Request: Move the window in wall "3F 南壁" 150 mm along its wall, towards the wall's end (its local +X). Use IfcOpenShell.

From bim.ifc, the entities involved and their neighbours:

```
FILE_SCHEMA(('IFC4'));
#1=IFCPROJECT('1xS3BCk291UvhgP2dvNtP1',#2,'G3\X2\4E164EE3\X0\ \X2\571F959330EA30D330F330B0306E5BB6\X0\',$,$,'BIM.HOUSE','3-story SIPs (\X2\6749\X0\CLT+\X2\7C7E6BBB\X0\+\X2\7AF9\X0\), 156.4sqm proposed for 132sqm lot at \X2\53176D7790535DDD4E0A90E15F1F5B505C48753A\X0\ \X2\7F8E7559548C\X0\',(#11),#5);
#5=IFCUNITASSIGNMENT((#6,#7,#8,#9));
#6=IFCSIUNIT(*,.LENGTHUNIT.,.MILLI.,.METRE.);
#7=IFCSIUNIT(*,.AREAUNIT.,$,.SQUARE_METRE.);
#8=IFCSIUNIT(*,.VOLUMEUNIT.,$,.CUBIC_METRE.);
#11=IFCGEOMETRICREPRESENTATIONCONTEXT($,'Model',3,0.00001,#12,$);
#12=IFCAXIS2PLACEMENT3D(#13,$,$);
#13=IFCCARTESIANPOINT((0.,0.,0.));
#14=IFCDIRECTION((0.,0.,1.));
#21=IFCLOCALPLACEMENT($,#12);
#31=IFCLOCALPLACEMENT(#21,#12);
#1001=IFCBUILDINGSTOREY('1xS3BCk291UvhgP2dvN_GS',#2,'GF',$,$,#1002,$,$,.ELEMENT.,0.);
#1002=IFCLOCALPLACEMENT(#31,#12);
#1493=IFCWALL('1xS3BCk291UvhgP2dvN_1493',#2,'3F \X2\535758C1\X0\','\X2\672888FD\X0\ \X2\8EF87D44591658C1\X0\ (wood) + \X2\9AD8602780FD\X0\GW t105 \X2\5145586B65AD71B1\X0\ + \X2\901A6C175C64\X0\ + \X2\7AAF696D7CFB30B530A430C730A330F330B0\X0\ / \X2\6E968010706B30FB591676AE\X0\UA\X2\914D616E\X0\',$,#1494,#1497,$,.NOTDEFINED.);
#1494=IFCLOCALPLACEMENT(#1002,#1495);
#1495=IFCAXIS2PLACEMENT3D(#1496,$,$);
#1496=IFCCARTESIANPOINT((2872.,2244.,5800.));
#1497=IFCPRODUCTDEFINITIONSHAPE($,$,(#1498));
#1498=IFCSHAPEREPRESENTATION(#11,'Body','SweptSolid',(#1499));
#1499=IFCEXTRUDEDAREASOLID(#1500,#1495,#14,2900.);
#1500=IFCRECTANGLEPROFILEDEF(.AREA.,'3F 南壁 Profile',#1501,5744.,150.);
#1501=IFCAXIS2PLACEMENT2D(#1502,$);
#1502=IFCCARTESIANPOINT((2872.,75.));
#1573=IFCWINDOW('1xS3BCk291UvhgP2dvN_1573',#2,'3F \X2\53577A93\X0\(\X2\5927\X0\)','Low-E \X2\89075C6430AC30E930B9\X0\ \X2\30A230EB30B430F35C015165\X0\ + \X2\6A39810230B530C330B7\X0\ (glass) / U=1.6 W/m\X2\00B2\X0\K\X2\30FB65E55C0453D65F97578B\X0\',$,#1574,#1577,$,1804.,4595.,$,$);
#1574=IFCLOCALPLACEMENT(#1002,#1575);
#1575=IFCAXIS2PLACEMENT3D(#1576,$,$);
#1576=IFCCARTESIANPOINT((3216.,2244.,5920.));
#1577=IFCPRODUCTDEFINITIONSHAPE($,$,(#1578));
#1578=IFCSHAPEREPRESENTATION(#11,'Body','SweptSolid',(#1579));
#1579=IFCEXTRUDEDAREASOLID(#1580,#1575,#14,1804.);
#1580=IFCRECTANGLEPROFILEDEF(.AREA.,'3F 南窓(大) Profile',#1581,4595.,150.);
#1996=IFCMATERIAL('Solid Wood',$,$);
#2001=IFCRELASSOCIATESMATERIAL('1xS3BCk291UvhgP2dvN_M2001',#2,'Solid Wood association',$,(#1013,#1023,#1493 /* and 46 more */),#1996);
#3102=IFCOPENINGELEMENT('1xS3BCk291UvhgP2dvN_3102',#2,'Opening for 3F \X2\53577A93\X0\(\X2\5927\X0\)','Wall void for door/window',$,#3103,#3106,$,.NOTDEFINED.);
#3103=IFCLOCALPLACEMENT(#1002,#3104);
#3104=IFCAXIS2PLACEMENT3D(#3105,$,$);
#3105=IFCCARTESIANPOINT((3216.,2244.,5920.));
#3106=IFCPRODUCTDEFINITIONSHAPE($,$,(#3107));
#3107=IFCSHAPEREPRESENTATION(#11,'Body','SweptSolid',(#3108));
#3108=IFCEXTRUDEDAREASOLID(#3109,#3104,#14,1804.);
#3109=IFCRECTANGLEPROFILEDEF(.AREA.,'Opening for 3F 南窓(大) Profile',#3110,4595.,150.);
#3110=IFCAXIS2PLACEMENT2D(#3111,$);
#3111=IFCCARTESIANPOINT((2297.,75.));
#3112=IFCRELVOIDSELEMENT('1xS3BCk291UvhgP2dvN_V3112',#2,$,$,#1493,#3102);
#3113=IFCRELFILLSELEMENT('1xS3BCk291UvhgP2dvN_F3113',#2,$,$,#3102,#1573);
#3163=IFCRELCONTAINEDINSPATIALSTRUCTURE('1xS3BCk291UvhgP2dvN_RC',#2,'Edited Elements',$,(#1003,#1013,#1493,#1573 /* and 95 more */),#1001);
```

```python
import ifcopenshell
import ifcopenshell.api.geometry
import ifcopenshell.util.placement
import ifcopenshell.util.unit

model = ifcopenshell.open("bim.ifc")
unit_scale = ifcopenshell.util.unit.calculate_unit_scale(model)

window = model.by_guid("1xS3BCk291UvhgP2dvN_1573")
opening = window.FillsVoids[0].RelatingOpeningElement
wall = opening.VoidsElements[0].RelatingBuildingElement

wall_matrix = ifcopenshell.util.placement.get_local_placement(wall.ObjectPlacement)
shift = wall_matrix[:3, 0] * 0.15 / unit_scale
before = ifcopenshell.util.placement.get_local_placement(window.ObjectPlacement)[:3, 3].copy()

# The window is not placed relative to its opening, so move both.
for product in (opening, window):
    matrix = ifcopenshell.util.placement.get_local_placement(product.ObjectPlacement)
    matrix[:3, 3] += shift
    ifcopenshell.api.geometry.edit_object_placement(model, product=product, matrix=matrix, is_si=False)

after = ifcopenshell.util.placement.get_local_placement(window.ObjectPlacement)[:3, 3]
print("window moved by", (after - before).round(3) + 0.0)

model.write("bim-out.ifc")
```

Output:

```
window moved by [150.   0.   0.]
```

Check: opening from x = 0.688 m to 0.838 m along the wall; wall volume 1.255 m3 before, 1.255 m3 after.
